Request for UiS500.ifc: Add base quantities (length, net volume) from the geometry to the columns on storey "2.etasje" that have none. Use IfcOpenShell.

First a look at what the model holds.

```python
import ifcopenshell
import ifcopenshell.util.element
import ifcopenshell.util.unit

model = ifcopenshell.open("UiS500.ifc")
print(model.schema)
for unit_type in ("LENGTHUNIT", "AREAUNIT", "VOLUMEUNIT"):
    print(unit_type, ifcopenshell.util.unit.calculate_unit_scale(model, unit_type))
storey = next(s for s in model.by_type("IfcBuildingStorey") if s.Name == "2.etasje")
columns = [e for e in ifcopenshell.util.element.get_decomposition(storey) if e.is_a("IfcColumn")]
for e in sorted(columns, key=lambda e: e.id()):
    print(e.id(), e.is_a(), e.Name, list(ifcopenshell.util.element.get_psets(e, qtos_only=True)), sep=" | ")
```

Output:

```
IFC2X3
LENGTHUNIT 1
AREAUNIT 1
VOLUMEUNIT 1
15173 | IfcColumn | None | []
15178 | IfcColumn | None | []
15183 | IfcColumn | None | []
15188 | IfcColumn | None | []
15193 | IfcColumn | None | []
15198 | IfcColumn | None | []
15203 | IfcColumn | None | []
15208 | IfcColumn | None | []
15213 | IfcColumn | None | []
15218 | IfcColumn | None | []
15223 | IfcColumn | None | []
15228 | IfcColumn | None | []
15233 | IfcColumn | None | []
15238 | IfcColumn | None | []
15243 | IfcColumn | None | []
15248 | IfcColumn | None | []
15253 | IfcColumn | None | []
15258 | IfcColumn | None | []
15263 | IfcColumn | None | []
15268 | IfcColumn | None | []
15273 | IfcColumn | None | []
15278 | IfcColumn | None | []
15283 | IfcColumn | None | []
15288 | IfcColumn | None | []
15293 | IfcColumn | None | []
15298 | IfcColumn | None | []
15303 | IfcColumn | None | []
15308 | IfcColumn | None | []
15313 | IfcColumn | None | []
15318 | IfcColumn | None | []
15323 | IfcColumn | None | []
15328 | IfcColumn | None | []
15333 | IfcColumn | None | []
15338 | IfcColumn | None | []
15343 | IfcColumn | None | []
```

```python
import ifcopenshell
import ifcopenshell.api.pset
import ifcopenshell.geom
import ifcopenshell.util.element
import ifcopenshell.util.shape
import ifcopenshell.util.unit

model = ifcopenshell.open("UiS500.ifc")
unit_scale = ifcopenshell.util.unit.calculate_unit_scale(model)
volume_scale = ifcopenshell.util.unit.calculate_unit_scale(model, "VOLUMEUNIT")
settings = ifcopenshell.geom.settings()

storey = next(s for s in model.by_type("IfcBuildingStorey") if s.Name == "2.etasje")
columns = [e for e in ifcopenshell.util.element.get_decomposition(storey) if e.is_a("IfcColumn")]

for e in sorted(columns, key=lambda e: e.id()):
    if ifcopenshell.util.element.get_psets(e, qtos_only=True, should_inherit=False):
        continue
    # Geometry comes back in metres, in the element's own axes.
    shape = ifcopenshell.geom.create_shape(settings, e)
    values = {
        "Length": ifcopenshell.util.shape.get_z(shape.geometry) / unit_scale,
        "NetVolume": ifcopenshell.util.shape.get_volume(shape.geometry) / volume_scale,
    }
    qto = ifcopenshell.api.pset.add_qto(model, product=e, name="BaseQuantities")
    ifcopenshell.api.pset.edit_qto(model, qto=qto, properties=values)
    print(e.id(), {k: round(v, 3) for k, v in values.items()})

model.write("UiS500_v2.ifc")
```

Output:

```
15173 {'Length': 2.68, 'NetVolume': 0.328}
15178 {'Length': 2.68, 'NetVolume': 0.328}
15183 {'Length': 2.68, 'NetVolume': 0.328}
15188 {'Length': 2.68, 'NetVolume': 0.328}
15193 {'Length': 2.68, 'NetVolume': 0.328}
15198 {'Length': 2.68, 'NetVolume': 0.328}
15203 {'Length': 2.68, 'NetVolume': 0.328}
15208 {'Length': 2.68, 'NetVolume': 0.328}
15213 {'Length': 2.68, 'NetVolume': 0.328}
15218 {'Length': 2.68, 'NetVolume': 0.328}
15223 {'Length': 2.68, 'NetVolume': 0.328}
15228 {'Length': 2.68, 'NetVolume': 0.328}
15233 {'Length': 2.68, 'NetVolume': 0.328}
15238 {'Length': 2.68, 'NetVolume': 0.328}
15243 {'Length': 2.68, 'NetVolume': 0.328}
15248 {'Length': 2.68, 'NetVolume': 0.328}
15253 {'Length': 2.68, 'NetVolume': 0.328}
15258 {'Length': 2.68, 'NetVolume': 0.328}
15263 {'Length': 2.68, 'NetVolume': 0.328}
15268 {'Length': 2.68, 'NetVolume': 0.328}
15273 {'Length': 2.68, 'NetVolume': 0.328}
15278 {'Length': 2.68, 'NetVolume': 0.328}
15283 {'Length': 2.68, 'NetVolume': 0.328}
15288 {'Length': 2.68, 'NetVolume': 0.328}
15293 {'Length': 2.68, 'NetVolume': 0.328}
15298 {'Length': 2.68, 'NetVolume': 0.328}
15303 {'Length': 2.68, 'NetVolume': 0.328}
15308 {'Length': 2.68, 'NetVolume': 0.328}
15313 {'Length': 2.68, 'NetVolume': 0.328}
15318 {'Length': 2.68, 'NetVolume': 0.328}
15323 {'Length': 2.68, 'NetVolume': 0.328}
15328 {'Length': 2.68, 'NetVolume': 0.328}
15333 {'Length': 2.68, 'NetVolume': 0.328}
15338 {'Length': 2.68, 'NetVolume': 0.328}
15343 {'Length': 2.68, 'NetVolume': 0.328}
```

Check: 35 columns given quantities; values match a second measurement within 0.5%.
